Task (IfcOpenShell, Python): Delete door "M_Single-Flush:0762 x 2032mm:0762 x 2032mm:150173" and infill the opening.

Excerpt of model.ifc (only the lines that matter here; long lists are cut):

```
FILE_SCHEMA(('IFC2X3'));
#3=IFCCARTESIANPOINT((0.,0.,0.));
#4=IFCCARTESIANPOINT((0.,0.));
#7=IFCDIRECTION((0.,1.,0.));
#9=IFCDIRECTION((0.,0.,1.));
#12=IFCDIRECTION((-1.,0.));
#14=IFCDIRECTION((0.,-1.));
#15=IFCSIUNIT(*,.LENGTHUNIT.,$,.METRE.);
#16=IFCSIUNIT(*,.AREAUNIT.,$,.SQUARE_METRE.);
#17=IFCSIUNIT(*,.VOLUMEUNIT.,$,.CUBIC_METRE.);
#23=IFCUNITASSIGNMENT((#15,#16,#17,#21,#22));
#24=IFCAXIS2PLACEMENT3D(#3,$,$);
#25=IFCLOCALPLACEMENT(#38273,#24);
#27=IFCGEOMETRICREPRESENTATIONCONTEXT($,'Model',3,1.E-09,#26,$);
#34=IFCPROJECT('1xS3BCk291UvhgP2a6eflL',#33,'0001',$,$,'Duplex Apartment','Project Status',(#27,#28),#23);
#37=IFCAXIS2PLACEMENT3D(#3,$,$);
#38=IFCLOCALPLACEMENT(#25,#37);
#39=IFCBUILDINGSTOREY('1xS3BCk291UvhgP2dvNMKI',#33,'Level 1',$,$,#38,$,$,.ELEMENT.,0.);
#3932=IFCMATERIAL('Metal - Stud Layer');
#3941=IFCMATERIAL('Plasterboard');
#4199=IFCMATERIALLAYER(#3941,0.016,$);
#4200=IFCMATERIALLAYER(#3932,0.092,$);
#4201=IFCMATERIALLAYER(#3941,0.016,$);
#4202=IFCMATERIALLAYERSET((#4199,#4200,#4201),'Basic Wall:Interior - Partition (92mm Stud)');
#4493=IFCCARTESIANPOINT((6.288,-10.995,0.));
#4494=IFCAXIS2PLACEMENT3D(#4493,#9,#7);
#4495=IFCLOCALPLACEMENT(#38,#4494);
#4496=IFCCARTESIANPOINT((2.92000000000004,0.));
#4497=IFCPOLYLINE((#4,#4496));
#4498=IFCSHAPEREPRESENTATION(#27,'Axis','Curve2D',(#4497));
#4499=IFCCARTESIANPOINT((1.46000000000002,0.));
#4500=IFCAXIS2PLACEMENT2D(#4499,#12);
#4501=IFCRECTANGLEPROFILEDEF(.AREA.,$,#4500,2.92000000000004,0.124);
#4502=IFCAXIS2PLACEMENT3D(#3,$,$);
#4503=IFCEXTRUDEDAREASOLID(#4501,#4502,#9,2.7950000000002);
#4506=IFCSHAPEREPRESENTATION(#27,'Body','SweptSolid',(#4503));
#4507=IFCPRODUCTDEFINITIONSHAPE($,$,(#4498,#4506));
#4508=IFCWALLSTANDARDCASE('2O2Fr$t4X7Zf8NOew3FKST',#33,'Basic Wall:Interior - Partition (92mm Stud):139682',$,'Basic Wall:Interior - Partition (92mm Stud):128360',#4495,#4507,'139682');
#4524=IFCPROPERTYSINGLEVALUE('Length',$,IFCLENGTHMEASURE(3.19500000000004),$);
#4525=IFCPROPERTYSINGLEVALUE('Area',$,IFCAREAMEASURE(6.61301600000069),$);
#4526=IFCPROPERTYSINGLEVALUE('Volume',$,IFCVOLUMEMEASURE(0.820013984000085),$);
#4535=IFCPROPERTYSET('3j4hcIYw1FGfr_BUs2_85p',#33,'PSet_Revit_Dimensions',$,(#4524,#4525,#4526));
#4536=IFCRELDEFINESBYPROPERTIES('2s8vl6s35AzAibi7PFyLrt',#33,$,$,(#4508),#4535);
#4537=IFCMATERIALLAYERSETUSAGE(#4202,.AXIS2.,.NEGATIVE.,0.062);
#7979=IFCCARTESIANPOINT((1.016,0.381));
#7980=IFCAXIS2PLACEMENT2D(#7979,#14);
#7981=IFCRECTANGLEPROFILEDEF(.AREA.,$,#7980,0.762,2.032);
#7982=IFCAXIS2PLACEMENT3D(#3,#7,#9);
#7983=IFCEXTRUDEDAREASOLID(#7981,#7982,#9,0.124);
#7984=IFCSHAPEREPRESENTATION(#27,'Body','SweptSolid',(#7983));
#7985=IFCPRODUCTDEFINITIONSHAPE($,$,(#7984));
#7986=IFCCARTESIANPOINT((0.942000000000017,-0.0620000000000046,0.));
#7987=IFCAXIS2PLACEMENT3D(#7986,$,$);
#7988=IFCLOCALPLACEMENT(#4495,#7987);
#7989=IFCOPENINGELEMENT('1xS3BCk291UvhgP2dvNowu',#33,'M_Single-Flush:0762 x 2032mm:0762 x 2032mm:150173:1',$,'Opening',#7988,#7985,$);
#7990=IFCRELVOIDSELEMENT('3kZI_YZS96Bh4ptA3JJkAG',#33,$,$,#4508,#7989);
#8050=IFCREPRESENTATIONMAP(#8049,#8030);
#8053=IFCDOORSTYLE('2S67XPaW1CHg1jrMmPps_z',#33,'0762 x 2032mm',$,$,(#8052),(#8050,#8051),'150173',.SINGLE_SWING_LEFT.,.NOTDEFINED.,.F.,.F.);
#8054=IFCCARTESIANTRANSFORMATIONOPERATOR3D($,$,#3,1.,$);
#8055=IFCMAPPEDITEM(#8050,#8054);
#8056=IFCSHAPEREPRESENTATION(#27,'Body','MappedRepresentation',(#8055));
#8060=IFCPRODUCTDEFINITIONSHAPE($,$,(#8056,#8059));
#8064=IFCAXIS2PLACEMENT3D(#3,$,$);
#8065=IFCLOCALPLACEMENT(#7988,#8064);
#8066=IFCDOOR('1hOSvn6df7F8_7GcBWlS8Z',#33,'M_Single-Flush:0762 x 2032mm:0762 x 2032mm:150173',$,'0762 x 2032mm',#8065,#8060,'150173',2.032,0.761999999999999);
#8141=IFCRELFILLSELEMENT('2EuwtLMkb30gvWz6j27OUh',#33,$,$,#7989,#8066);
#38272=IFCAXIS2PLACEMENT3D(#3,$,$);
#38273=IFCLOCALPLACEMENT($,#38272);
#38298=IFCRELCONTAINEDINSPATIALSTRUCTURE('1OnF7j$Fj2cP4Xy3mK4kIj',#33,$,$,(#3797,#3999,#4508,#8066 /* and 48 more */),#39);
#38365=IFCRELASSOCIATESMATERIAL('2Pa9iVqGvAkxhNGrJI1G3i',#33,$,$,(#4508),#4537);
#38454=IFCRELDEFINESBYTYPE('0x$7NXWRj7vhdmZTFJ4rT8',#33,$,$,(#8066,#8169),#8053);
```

```python
import ifcopenshell
import ifcopenshell.api.feature
import ifcopenshell.api.pset
import ifcopenshell.api.root
import ifcopenshell.geom
import ifcopenshell.util.element
import ifcopenshell.util.shape
import ifcopenshell.util.unit

model = ifcopenshell.open("model.ifc")
area_scale = ifcopenshell.util.unit.calculate_unit_scale(model, "AREAUNIT")
volume_scale = ifcopenshell.util.unit.calculate_unit_scale(model, "VOLUMEUNIT")
settings = ifcopenshell.geom.settings()


def volume(element):
    """Net volume in cubic metres, openings subtracted."""
    shape = ifcopenshell.geom.create_shape(settings, element)
    return ifcopenshell.util.shape.get_volume(shape.geometry)


door = model.by_guid("1hOSvn6df7F8_7GcBWlS8Z")
opening = door.FillsVoids[0].RelatingOpeningElement
wall = opening.VoidsElements[0].RelatingBuildingElement
before = volume(wall)

ifcopenshell.api.root.remove_product(model, product=door)
ifcopenshell.api.feature.remove_feature(model, feature=opening)

after = volume(wall)
thickness = 0.124  # wall thickness in metres

# Update the wall's stored quantities.
pset = model.by_id(ifcopenshell.util.element.get_pset(wall, "PSet_Revit_Dimensions", should_inherit=False)["id"])
ifcopenshell.api.pset.edit_pset(model, pset=pset, properties={
    "Area": model.create_entity("IfcAreaMeasure", after / thickness / area_scale),
    "Volume": model.create_entity("IfcVolumeMeasure", after / volume_scale),
})

print(f"wall volume {before:.3f} -> {after:.3f} m3")

model.write("model-out.ifc")
```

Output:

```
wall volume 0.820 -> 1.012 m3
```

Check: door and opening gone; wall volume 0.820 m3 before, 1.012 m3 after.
